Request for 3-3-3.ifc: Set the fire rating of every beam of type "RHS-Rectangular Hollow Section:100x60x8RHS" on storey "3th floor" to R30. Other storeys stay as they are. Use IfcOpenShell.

First a look at what the model holds.

```python
import ifcopenshell
import ifcopenshell.util.element

model = ifcopenshell.open("3-3-3.ifc")
print(model.schema)
storey = next(s for s in model.by_type("IfcBuildingStorey") if s.Name == "3th floor")
beams = [e for e in ifcopenshell.util.element.get_decomposition(storey) if e.is_a("IfcBeam")]
seen = {}
for e in beams:
    element_type = ifcopenshell.util.element.get_type(e)
    key = (element_type.Name if element_type != e and element_type else None, ifcopenshell.util.element.get_pset(e, "Pset_BeamCommon", "FireRating"))
    seen[key] = seen.get(key, 0) + 1
for (name, value), count in sorted(seen.items(), key=str):
    print(count, "x", name, "|", value)
```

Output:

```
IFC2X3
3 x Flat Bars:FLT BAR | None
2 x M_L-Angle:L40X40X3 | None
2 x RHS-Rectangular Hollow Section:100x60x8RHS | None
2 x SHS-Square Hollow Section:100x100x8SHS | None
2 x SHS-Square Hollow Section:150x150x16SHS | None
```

```python
import ifcopenshell
import ifcopenshell.api.pset
import ifcopenshell.util.element

model = ifcopenshell.open("3-3-3.ifc")

storey = next(s for s in model.by_type("IfcBuildingStorey") if s.Name == "3th floor")
beams = [e for e in ifcopenshell.util.element.get_decomposition(storey) if e.is_a("IfcBeam")]

count = 0
for e in beams:
    element_type = ifcopenshell.util.element.get_type(e)
    if element_type in (None, e) or element_type.Name != "RHS-Rectangular Hollow Section:100x60x8RHS":
        continue
    # add_pset returns the element's existing set when there is one.
    pset = ifcopenshell.api.pset.add_pset(model, product=e, name="Pset_BeamCommon")
    ifcopenshell.api.pset.edit_pset(model, pset=pset, properties={"FireRating": "R30"})
    count += 1

print(count, "beams updated")

model.write("3-3-3_edited.ifc")
```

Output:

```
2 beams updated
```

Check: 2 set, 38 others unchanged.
